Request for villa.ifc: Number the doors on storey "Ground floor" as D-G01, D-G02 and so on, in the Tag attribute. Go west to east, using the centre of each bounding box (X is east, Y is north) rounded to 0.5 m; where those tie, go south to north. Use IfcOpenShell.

First a look at what the model holds.

```python
import ifcopenshell
import ifcopenshell.util.element
import ifcopenshell.util.placement

model = ifcopenshell.open("villa.ifc")
print(model.schema)
storey = next(s for s in model.by_type("IfcBuildingStorey") if s.Name == "Ground floor")
doors = [e for e in ifcopenshell.util.element.get_decomposition(storey) if e.is_a("IfcDoor")]
for e in sorted(doors, key=lambda e: e.id()):
    origin = ifcopenshell.util.placement.get_local_placement(e.ObjectPlacement)[:3, 3]
    print(e.id(), e.Tag, e.Name, origin.round(2) + 0.0, sep=" | ")
```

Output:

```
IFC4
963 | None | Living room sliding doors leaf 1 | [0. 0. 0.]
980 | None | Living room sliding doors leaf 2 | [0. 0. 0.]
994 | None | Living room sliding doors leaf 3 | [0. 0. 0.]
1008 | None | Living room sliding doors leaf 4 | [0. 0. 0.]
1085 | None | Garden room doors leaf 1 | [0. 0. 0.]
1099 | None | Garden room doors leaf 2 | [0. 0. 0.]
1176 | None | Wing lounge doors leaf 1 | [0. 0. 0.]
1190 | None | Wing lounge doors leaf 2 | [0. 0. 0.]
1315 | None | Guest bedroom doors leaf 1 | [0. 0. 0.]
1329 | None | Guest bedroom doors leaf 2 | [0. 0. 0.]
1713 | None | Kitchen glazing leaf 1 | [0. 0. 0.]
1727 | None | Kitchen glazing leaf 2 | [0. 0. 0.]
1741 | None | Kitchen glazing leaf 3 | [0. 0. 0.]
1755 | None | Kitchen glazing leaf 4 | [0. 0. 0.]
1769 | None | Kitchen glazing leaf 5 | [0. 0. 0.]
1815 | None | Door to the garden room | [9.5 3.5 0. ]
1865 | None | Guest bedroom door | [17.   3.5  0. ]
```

```python
import ifcopenshell
import ifcopenshell.geom
import ifcopenshell.util.element
import ifcopenshell.util.shape

model = ifcopenshell.open("villa.ifc")
settings = ifcopenshell.geom.settings()
settings.set("use-world-coords", True)


def centre(element):
    shape = ifcopenshell.geom.create_shape(settings, element)
    return ifcopenshell.util.shape.get_bbox_centroid(shape.geometry)


storey = next(s for s in model.by_type("IfcBuildingStorey") if s.Name == "Ground floor")
doors = [e for e in ifcopenshell.util.element.get_decomposition(storey) if e.is_a("IfcDoor")]

# Insertion points can sit at a corner or the storey origin, so sort by the geometry (in metres).
centres = {e: centre(e) for e in doors}
doors.sort(key=lambda e: (round(centres[e][0] / 0.5), centres[e][1]))

for i, e in enumerate(doors, start=1):
    number = f"D-G{i:02d}"
    e.Tag = number
    print(e.id(), number)

model.write("villa_updated.ifc")
```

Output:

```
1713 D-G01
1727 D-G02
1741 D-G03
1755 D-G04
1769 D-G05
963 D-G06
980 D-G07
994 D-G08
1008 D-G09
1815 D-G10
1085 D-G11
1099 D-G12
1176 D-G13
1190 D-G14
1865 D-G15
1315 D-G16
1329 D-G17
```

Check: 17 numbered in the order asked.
